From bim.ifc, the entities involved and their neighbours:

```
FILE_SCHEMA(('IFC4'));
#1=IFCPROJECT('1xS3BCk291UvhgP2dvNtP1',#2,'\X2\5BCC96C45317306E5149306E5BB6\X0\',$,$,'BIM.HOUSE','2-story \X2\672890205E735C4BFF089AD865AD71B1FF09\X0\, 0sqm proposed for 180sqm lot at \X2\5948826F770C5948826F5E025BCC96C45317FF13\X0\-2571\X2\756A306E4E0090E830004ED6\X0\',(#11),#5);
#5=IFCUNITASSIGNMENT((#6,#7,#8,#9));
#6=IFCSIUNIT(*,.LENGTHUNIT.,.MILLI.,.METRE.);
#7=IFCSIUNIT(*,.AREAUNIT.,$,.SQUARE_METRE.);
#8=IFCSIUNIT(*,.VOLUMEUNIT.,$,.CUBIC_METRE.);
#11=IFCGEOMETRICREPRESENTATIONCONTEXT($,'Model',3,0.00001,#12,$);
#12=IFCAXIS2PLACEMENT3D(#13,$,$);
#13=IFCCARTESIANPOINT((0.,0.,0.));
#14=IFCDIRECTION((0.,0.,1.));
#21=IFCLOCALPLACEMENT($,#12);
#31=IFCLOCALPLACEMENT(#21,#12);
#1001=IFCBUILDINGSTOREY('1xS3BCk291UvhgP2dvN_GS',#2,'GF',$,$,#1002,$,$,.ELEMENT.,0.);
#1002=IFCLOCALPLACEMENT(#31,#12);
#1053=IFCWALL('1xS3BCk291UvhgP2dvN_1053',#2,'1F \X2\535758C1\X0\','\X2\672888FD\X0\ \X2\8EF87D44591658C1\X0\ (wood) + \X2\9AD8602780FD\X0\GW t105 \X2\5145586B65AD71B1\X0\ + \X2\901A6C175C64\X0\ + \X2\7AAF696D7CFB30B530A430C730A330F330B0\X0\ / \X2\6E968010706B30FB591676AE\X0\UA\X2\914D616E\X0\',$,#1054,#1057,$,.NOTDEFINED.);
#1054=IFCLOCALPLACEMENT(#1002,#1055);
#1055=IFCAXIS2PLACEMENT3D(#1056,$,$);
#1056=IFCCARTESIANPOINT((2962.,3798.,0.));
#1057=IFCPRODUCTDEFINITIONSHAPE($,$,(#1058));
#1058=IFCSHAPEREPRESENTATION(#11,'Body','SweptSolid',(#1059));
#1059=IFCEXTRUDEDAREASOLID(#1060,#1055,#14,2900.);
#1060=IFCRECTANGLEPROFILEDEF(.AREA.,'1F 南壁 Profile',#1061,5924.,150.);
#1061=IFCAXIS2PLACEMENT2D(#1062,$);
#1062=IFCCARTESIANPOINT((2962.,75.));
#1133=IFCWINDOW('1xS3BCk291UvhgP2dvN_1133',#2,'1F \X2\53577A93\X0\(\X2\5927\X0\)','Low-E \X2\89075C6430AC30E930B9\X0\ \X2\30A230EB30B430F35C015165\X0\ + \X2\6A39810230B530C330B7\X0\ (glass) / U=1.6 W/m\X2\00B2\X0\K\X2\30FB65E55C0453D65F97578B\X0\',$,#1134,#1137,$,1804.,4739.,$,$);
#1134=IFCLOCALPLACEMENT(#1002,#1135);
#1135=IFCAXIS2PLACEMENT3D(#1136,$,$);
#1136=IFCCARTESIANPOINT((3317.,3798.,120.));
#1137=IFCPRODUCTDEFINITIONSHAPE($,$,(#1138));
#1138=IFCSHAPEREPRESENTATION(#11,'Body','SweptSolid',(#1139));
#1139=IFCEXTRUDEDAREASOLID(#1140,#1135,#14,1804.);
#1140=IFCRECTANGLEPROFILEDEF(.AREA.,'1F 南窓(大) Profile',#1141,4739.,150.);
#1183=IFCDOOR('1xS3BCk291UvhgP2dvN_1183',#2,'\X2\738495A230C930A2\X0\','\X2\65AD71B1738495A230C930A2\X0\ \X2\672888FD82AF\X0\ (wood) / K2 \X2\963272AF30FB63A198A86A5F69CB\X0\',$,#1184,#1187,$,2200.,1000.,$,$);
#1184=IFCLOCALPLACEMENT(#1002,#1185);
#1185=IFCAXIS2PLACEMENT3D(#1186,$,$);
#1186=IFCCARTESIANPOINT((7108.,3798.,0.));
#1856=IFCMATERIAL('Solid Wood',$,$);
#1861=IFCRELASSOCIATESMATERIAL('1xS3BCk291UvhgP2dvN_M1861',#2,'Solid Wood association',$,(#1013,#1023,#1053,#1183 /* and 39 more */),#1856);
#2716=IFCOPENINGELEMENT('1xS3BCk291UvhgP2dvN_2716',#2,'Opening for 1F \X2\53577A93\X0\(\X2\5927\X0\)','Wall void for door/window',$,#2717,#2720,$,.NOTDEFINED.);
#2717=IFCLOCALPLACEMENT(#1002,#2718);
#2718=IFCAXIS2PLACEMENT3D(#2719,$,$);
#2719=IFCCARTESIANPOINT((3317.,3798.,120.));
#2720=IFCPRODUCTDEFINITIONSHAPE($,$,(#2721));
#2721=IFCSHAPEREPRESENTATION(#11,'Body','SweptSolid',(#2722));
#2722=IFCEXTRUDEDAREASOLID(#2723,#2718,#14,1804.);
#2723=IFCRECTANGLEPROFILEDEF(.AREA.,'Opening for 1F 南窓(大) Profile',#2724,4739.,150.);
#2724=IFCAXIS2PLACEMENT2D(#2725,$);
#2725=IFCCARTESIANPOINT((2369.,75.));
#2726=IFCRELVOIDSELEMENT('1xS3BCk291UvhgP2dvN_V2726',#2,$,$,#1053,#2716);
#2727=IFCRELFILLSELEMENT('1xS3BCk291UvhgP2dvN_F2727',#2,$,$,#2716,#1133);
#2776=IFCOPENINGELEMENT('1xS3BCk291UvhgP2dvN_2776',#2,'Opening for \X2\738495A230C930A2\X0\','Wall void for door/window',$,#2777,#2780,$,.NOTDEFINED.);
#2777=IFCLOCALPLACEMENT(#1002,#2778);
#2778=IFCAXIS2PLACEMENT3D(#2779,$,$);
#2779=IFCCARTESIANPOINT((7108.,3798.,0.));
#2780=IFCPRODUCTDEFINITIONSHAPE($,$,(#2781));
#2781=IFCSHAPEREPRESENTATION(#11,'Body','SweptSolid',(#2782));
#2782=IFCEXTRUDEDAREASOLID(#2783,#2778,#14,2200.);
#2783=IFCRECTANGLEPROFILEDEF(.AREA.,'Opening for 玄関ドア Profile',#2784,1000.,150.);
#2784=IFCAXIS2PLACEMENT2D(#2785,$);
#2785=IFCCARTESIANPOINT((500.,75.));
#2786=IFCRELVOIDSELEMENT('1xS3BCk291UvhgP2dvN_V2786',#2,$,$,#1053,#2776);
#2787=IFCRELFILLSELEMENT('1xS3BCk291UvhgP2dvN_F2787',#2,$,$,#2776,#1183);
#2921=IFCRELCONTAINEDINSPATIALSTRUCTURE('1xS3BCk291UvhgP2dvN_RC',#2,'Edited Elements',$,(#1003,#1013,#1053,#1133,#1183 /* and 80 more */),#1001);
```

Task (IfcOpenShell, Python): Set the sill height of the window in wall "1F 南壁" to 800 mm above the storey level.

```python
import numpy as np
import ifcopenshell
import ifcopenshell.api.geometry
import ifcopenshell.geom
import ifcopenshell.util.element
import ifcopenshell.util.placement
import ifcopenshell.util.shape
import ifcopenshell.util.unit

model = ifcopenshell.open("bim.ifc")
unit_scale = ifcopenshell.util.unit.calculate_unit_scale(model)

window = model.by_id(1133)
opening = window.FillsVoids[0].RelatingOpeningElement
storey = ifcopenshell.util.element.get_container(window, ifc_class="IfcBuildingStorey")
level = ifcopenshell.util.placement.get_local_placement(storey.ObjectPlacement)[2, 3]

# The opening's origin need not be at the sill, so measure its lowest point.
shape = ifcopenshell.geom.create_shape(ifcopenshell.geom.settings(), opening)
bottom = ifcopenshell.util.shape.get_shape_bottom_elevation(shape, shape.geometry) / unit_scale
dz = level + 0.8 / unit_scale - bottom

shift = np.array([0.0, 0.0, dz])
# The window is not placed relative to its opening, so move both.
for product in (opening, window):
    matrix = ifcopenshell.util.placement.get_local_placement(product.ObjectPlacement)
    matrix[:3, 3] += shift
    ifcopenshell.api.geometry.edit_object_placement(model, product=product, matrix=matrix, is_si=False)

print(f"moved by {dz * unit_scale:+.3f} m")

model.write("bim-out.ifc")
```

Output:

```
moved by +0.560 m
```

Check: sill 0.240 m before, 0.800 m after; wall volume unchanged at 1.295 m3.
